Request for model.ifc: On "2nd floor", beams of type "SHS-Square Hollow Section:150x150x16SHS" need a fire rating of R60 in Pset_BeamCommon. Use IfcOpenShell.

First a look at what the model holds.

```python
import ifcopenshell
import ifcopenshell.util.element

model = ifcopenshell.open("model.ifc")
print(model.schema)
storey = next(s for s in model.by_type("IfcBuildingStorey") if s.Name == "2nd floor")
beams = [e for e in ifcopenshell.util.element.get_decomposition(storey) if e.is_a("IfcBeam")]
seen = {}
for e in beams:
    element_type = ifcopenshell.util.element.get_type(e)
    key = (element_type.Name if element_type != e and element_type else None, ifcopenshell.util.element.get_pset(e, "Pset_BeamCommon", "FireRating"))
    seen[key] = seen.get(key, 0) + 1
for (name, value), count in sorted(seen.items(), key=str):
    print(count, "x", name, "|", value)
```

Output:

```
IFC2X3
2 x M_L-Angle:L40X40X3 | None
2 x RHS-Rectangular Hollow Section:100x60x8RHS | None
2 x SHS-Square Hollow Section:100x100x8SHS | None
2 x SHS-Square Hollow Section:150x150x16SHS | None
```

```python
import ifcopenshell
import ifcopenshell.api.pset
import ifcopenshell.util.element

model = ifcopenshell.open("model.ifc")

storey = next(s for s in model.by_type("IfcBuildingStorey") if s.Name == "2nd floor")
beams = [e for e in ifcopenshell.util.element.get_decomposition(storey) if e.is_a("IfcBeam")]

count = 0
for e in beams:
    element_type = ifcopenshell.util.element.get_type(e)
    if element_type in (None, e) or element_type.Name != "SHS-Square Hollow Section:150x150x16SHS":
        continue
    # add_pset returns the element's existing set when there is one.
    pset = ifcopenshell.api.pset.add_pset(model, product=e, name="Pset_BeamCommon")
    ifcopenshell.api.pset.edit_pset(model, pset=pset, properties={"FireRating": "R60"})
    count += 1

print(count, "beams updated")

model.write("model_edited.ifc")
```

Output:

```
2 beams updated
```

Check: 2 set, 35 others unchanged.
